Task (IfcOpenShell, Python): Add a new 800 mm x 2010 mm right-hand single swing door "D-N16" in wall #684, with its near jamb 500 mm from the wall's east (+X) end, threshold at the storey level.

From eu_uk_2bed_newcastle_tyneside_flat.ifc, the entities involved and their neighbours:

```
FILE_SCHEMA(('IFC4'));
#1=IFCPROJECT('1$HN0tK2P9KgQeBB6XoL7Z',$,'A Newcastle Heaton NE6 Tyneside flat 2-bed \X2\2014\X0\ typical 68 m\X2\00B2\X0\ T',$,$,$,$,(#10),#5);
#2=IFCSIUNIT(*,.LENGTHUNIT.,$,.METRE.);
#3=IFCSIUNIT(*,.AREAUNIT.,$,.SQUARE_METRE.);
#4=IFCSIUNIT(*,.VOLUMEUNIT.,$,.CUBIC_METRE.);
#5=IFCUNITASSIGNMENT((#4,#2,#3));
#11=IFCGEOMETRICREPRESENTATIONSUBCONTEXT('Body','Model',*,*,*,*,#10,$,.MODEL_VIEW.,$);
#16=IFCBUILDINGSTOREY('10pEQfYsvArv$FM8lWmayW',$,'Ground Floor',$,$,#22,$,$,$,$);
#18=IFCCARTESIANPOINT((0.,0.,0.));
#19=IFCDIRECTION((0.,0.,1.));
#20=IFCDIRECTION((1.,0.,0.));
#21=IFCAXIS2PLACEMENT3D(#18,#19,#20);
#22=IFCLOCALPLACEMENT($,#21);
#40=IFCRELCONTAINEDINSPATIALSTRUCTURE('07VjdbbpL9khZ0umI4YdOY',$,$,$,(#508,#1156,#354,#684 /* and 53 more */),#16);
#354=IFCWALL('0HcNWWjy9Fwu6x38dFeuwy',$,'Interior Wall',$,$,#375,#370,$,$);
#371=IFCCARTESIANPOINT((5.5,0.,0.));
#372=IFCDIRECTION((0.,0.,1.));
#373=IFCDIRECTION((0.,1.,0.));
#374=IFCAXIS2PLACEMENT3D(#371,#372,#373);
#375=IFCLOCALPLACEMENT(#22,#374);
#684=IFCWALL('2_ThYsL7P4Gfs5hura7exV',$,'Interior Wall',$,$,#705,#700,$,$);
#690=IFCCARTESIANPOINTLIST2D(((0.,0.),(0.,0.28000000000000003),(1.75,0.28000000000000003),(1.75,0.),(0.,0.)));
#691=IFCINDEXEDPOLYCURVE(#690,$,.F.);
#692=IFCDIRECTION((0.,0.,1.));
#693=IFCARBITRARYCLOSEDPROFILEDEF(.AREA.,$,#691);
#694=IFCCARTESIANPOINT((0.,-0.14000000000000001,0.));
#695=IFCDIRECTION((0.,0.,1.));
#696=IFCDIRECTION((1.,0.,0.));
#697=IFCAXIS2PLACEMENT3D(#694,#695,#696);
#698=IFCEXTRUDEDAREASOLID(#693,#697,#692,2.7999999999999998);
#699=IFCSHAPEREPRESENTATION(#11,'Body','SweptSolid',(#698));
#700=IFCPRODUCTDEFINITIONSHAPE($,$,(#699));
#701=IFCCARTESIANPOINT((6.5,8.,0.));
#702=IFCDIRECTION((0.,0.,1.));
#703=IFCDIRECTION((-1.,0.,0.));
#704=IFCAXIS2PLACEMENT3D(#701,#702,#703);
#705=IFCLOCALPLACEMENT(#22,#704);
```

```python
import numpy as np
import ifcopenshell
import ifcopenshell.api.feature
import ifcopenshell.api.geometry
import ifcopenshell.api.root
import ifcopenshell.api.spatial
import ifcopenshell.geom
import ifcopenshell.util.element
import ifcopenshell.util.placement
import ifcopenshell.util.representation
import ifcopenshell.util.shape
import ifcopenshell.util.unit

model = ifcopenshell.open("eu_uk_2bed_newcastle_tyneside_flat.ifc")
unit_scale = ifcopenshell.util.unit.calculate_unit_scale(model)
settings = ifcopenshell.geom.settings()


def volume(element):
    """Net volume in cubic metres, openings subtracted."""
    shape = ifcopenshell.geom.create_shape(settings, element)
    return ifcopenshell.util.shape.get_volume(shape.geometry)


wall = model.by_guid("2_ThYsL7P4Gfs5hura7exV")
storey = ifcopenshell.util.element.get_container(wall, ifc_class="IfcBuildingStorey")
context = ifcopenshell.util.representation.get_context(model, "Model", "Body", "MODEL_VIEW")
before = volume(wall)

width, height, from_end, sill = 0.8, 2.01, 0.5, 0.0  # metres

# The wall runs along its own X axis, and the end named is its -X end.
wall_shape = ifcopenshell.geom.create_shape(settings, wall)
x, y, z = ifcopenshell.util.shape.get_vertices(wall_shape.geometry).T
start = x.min() + from_end
face, thickness = float(y.min()), float(y.max() - y.min())
wall_matrix = ifcopenshell.util.placement.get_local_placement(wall.ObjectPlacement)
level = ifcopenshell.util.placement.get_local_placement(storey.ObjectPlacement)[2, 3]


def in_wall(x, y):
    """Placement at x, y metres in the wall's axes, at sill height."""
    matrix = wall_matrix.copy()
    matrix[:, 3] = wall_matrix @ np.array([x / unit_scale, y / unit_scale, 0.0, 1.0])
    matrix[2, 3] = level + sill / unit_scale
    return matrix


# Opening: a box that overshoots both wall faces by 50 mm.
opening = ifcopenshell.api.root.create_entity(model, ifc_class="IfcOpeningElement", predefined_type="OPENING")
box = ifcopenshell.api.geometry.add_wall_representation(
    model, context=context, length=width, height=height, thickness=thickness + 0.1
)
ifcopenshell.api.geometry.assign_representation(model, product=opening, representation=box)
ifcopenshell.api.geometry.edit_object_placement(model, product=opening, matrix=in_wall(start, face - 0.05), is_si=False)
ifcopenshell.api.feature.add_feature(model, feature=opening, element=wall)

door = ifcopenshell.api.root.create_entity(model, ifc_class="IfcDoor", name="D-N16", predefined_type="DOOR")
door.OverallWidth, door.OverallHeight = width / unit_scale, height / unit_scale
door.OperationType = "SINGLE_SWING_RIGHT"
body = ifcopenshell.api.geometry.add_door_representation(
    model,
    context=context,
    overall_width=door.OverallWidth,
    overall_height=door.OverallHeight,
    operation_type="SINGLE_SWING_RIGHT",
    lining_properties={"LiningDepth": thickness / unit_scale, "ThresholdDepth": thickness / unit_scale},
)
ifcopenshell.api.geometry.assign_representation(model, product=door, representation=body)
ifcopenshell.api.spatial.assign_container(model, products=[door], relating_structure=storey)
ifcopenshell.api.feature.add_filling(model, opening=opening, element=door)

# The lining spans the wall, so the door starts at the wall face.
ifcopenshell.api.geometry.edit_object_placement(model, product=door, matrix=in_wall(start, face), is_si=False)

after = volume(wall)

print(f"wall volume {before:.3f} -> {after:.3f} m3")

model.write("eu_uk_2bed_newcastle_tyneside_flat_edited.ifc")
```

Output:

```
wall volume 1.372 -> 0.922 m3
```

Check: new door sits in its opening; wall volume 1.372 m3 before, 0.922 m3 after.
